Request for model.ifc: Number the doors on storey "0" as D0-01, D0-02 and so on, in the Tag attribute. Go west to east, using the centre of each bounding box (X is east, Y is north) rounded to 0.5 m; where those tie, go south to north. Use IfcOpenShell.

First a look at what the model holds.

```python
import ifcopenshell
import ifcopenshell.util.element
import ifcopenshell.util.placement

model = ifcopenshell.open("model.ifc")
print(model.schema)
storey = next(s for s in model.by_type("IfcBuildingStorey") if s.Name == "0")
doors = [e for e in ifcopenshell.util.element.get_decomposition(storey) if e.is_a("IfcDoor")]
for e in sorted(doors, key=lambda e: e.id()):
    origin = ifcopenshell.util.placement.get_local_placement(e.ObjectPlacement)[:3, 3]
    print(e.id(), e.Tag, e.Name, origin.round(2) + 0.0, sep=" | ")
```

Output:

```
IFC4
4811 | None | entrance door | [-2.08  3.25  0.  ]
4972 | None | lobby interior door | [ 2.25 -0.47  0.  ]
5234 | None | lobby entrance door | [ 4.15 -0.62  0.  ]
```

```python
import ifcopenshell
import ifcopenshell.geom
import ifcopenshell.util.element
import ifcopenshell.util.shape

model = ifcopenshell.open("model.ifc")
settings = ifcopenshell.geom.settings()
settings.set("use-world-coords", True)


def centre(element):
    shape = ifcopenshell.geom.create_shape(settings, element)
    return ifcopenshell.util.shape.get_bbox_centroid(shape.geometry)


storey = next(s for s in model.by_type("IfcBuildingStorey") if s.Name == "0")
doors = [e for e in ifcopenshell.util.element.get_decomposition(storey) if e.is_a("IfcDoor")]

# Insertion points can sit at a corner or the storey origin, so sort by the geometry (in metres).
centres = {e: centre(e) for e in doors}
doors.sort(key=lambda e: (round(centres[e][0] / 0.5), centres[e][1]))

for i, e in enumerate(doors, start=1):
    number = f"D0-{i:02d}"
    e.Tag = number
    print(e.id(), number)

model.write("model_v2.ifc")
```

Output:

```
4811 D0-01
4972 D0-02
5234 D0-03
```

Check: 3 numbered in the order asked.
